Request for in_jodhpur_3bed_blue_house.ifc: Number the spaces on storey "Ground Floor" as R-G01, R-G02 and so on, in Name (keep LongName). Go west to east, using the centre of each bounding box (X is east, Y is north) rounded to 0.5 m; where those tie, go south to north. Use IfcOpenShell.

First a look at what the model holds.

```python
import ifcopenshell
import ifcopenshell.util.element
import ifcopenshell.util.placement

model = ifcopenshell.open("in_jodhpur_3bed_blue_house.ifc")
print(model.schema)
storey = next(s for s in model.by_type("IfcBuildingStorey") if s.Name == "Ground Floor")
spaces = [e for e in ifcopenshell.util.element.get_decomposition(storey) if e.is_a("IfcSpace")]
for e in sorted(spaces, key=lambda e: e.id()):
    origin = ifcopenshell.util.placement.get_local_placement(e.ObjectPlacement)[:3, 3]
    print(e.id(), e.Name, e.LongName, origin.round(2) + 0.0, sep=" | ")
```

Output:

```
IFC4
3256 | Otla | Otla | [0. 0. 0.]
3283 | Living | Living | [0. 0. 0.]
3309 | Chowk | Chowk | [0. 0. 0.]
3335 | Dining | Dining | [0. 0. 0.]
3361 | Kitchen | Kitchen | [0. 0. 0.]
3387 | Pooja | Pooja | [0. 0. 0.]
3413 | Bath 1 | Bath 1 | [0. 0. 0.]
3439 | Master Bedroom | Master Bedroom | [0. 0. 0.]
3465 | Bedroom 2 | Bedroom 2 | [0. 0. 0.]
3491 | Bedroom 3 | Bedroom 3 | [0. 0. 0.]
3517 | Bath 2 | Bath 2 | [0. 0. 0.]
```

```python
import ifcopenshell
import ifcopenshell.geom
import ifcopenshell.util.element
import ifcopenshell.util.shape

model = ifcopenshell.open("in_jodhpur_3bed_blue_house.ifc")
settings = ifcopenshell.geom.settings()
settings.set("use-world-coords", True)


def centre(element):
    shape = ifcopenshell.geom.create_shape(settings, element)
    return ifcopenshell.util.shape.get_bbox_centroid(shape.geometry)


storey = next(s for s in model.by_type("IfcBuildingStorey") if s.Name == "Ground Floor")
spaces = [e for e in ifcopenshell.util.element.get_decomposition(storey) if e.is_a("IfcSpace")]

# Insertion points can sit at a corner or the storey origin, so sort by the geometry (in metres).
centres = {e: centre(e) for e in spaces}
spaces.sort(key=lambda e: (round(centres[e][0] / 0.5), centres[e][1]))

for i, e in enumerate(spaces, start=1):
    number = f"R-G{i:02d}"
    e.Name = number
    print(e.id(), number)

model.write("in_jodhpur_3bed_blue_house_edited.ifc")
```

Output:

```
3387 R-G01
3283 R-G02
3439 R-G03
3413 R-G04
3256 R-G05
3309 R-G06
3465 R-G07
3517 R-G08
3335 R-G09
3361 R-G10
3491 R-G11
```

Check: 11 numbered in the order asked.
